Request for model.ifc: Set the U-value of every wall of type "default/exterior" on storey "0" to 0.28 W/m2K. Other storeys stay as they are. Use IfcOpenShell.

First a look at what the model holds.

```python
import ifcopenshell
import ifcopenshell.util.element

model = ifcopenshell.open("model.ifc")
print(model.schema)
storey = next(s for s in model.by_type("IfcBuildingStorey") if s.Name == "0")
walls = [e for e in ifcopenshell.util.element.get_decomposition(storey) if e.is_a("IfcWall")]
seen = {}
for e in walls:
    element_type = ifcopenshell.util.element.get_type(e)
    key = (element_type.Name if element_type != e and element_type else None, ifcopenshell.util.element.get_pset(e, "Pset_WallCommon", "ThermalTransmittance"))
    seen[key] = seen.get(key, 0) + 1
for (name, value), count in sorted(seen.items(), key=str):
    print(count, "x", name, "|", value)
```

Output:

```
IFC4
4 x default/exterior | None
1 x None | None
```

```python
import ifcopenshell
import ifcopenshell.api.pset
import ifcopenshell.util.element

model = ifcopenshell.open("model.ifc")

storey = next(s for s in model.by_type("IfcBuildingStorey") if s.Name == "0")
walls = [e for e in ifcopenshell.util.element.get_decomposition(storey) if e.is_a("IfcWall")]

count = 0
for e in walls:
    element_type = ifcopenshell.util.element.get_type(e)
    if element_type in (None, e) or element_type.Name != "default/exterior":
        continue
    # add_pset returns the element's existing set when there is one.
    pset = ifcopenshell.api.pset.add_pset(model, product=e, name="Pset_WallCommon")
    ifcopenshell.api.pset.edit_pset(model, pset=pset, properties={"ThermalTransmittance": 0.28})
    count += 1

print(count, "walls updated")

model.write("model-out.ifc")
```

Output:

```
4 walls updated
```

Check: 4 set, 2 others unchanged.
